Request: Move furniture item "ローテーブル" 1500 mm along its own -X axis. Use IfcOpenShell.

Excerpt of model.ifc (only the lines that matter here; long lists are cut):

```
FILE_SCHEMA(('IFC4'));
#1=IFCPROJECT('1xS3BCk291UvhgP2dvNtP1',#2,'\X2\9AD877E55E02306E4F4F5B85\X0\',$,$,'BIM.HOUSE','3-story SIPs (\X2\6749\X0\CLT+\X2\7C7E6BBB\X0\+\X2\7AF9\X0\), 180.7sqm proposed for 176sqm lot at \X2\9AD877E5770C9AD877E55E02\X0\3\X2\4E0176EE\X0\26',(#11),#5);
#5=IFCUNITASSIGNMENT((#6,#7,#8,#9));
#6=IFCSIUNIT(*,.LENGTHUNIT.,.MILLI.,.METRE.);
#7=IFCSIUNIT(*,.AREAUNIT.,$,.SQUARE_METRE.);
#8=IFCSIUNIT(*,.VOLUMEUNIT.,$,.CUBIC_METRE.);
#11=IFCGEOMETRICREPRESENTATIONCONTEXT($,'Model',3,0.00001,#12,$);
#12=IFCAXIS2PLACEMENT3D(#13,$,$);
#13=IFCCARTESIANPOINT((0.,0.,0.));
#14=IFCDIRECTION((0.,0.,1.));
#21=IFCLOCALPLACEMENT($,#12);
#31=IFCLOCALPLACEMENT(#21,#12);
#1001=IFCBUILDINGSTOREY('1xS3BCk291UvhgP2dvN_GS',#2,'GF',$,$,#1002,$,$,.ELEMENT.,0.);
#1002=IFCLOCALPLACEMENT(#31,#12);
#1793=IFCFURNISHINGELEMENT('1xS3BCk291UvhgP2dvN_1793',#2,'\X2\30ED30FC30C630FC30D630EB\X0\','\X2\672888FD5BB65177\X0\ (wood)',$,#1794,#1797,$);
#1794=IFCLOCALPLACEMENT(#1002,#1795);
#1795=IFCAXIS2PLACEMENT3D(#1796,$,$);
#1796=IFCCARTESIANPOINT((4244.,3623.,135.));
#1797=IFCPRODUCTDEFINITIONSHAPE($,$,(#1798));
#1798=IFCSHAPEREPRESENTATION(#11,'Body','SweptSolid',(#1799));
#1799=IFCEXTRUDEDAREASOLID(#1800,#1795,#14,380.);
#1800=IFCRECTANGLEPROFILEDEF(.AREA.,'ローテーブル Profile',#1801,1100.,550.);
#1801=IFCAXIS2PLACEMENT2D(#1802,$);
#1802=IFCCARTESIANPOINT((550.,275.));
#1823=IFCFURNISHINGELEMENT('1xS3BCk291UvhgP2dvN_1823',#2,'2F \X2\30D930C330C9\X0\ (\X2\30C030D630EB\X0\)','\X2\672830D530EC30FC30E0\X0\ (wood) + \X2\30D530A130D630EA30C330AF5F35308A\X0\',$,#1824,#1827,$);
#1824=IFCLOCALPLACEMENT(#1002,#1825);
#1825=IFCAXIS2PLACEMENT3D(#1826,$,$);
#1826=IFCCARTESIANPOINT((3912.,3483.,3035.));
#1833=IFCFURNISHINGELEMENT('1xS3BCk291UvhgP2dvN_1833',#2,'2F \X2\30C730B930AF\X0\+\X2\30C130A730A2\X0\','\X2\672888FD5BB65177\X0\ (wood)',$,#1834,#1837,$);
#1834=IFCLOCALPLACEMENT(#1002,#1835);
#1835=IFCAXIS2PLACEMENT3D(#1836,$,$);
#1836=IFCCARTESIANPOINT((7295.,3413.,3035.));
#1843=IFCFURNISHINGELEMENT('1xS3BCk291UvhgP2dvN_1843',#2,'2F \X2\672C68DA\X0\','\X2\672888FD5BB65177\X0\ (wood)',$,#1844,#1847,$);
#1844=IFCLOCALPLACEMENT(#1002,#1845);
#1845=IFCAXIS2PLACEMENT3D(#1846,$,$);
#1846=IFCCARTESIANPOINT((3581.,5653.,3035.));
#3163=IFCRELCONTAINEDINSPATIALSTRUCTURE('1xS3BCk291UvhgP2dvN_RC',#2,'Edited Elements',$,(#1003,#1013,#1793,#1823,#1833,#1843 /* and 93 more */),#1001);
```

```python
import ifcopenshell
import ifcopenshell.api.geometry
import ifcopenshell.util.placement
import ifcopenshell.util.unit

model = ifcopenshell.open("model.ifc")
unit_scale = ifcopenshell.util.unit.calculate_unit_scale(model)

item = model.by_id(1793)
matrix = ifcopenshell.util.placement.get_local_placement(item.ObjectPlacement)
matrix[:3, 3] -= matrix[:3, 0] * 1.5 / unit_scale
ifcopenshell.api.geometry.edit_object_placement(model, product=item, matrix=matrix, is_si=False)

print(ifcopenshell.util.placement.get_local_placement(item.ObjectPlacement).round(3) + 0.0)

model.write("model_edited.ifc")
```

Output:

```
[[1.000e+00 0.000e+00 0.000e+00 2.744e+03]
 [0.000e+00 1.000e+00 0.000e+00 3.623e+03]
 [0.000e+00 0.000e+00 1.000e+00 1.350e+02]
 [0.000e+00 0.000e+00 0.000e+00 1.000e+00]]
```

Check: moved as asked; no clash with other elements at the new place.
